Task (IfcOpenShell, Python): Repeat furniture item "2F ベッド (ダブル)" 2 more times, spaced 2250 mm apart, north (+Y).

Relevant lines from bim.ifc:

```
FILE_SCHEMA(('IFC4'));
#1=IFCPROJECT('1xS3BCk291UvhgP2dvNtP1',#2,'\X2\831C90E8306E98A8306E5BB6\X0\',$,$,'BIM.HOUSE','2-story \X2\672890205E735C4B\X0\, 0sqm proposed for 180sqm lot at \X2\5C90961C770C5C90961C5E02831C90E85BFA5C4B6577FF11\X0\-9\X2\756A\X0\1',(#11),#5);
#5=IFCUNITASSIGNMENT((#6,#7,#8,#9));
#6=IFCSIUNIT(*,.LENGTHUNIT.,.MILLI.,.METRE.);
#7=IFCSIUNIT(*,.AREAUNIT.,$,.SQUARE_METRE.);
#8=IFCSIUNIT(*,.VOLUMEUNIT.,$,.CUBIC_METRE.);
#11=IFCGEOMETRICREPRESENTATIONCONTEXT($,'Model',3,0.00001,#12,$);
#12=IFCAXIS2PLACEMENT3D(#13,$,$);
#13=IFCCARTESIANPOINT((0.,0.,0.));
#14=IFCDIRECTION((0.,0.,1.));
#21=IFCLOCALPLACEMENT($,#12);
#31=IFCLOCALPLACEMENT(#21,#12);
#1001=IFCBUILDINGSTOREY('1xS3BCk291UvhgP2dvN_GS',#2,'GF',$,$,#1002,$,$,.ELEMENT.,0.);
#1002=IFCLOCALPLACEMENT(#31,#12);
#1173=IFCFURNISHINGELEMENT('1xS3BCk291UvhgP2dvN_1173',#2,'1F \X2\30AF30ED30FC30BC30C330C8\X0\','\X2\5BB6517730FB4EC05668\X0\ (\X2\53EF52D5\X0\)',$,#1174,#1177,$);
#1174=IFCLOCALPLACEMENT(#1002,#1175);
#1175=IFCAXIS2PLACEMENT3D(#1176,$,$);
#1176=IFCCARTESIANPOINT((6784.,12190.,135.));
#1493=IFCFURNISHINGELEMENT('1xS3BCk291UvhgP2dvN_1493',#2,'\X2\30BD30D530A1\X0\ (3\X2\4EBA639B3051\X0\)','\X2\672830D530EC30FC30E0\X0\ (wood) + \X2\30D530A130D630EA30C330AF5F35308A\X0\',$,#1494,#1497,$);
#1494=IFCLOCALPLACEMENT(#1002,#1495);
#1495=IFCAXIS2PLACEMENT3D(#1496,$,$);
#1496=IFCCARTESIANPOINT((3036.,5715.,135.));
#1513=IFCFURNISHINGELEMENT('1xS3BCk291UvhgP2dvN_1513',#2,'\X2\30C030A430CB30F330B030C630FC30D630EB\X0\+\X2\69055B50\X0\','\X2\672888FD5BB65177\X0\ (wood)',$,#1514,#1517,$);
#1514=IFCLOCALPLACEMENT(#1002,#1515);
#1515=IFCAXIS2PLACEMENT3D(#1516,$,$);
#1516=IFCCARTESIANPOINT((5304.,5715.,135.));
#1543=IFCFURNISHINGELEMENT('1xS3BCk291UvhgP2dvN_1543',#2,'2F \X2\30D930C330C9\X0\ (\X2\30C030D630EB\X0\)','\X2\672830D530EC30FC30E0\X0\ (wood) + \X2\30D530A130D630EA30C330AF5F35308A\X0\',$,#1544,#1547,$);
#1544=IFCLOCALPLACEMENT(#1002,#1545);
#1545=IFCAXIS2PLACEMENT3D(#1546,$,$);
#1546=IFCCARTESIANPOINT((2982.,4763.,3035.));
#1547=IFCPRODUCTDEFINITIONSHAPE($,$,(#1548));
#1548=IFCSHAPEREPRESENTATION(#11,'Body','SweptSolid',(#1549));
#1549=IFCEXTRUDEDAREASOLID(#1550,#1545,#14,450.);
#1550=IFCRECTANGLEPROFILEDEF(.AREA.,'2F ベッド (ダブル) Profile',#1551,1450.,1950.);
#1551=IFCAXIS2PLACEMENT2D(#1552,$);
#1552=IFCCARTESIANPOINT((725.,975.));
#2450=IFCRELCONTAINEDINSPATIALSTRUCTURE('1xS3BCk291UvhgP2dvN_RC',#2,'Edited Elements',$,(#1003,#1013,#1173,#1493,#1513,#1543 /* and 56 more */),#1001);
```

```python
import numpy as np
import ifcopenshell
import ifcopenshell.api.geometry
import ifcopenshell.api.root
import ifcopenshell.util.element
import ifcopenshell.util.placement
import ifcopenshell.util.unit

model = ifcopenshell.open("bim.ifc")
unit_scale = ifcopenshell.util.unit.calculate_unit_scale(model)


def reuse_history(source, copy):
    """copy_class also copies each property set's owner history, people and application; keep the originals."""
    for rel in copy.IsDefinedBy:
        if rel.is_a("IfcRelDefinesByProperties") and (history := rel.RelatingPropertyDefinition.OwnerHistory):
            rel.RelatingPropertyDefinition.OwnerHistory = source.OwnerHistory
            ifcopenshell.util.element.remove_deep2(model, history)


source = model.by_guid("1xS3BCk291UvhgP2dvN_1543")
base = ifcopenshell.util.placement.get_local_placement(source.ObjectPlacement)
step = np.array([0.0, 1.0, 0.0]) * 2.25 / unit_scale

for i in range(1, 3):
    copy = ifcopenshell.api.root.copy_class(model, product=source)
    copy.Representation = ifcopenshell.util.element.copy_deep(
        model, source.Representation, exclude=["IfcGeometricRepresentationContext", "IfcRepresentationMap"]
    )
    reuse_history(source, copy)
    matrix = base.copy()
    matrix[:3, 3] += i * step
    print("added at", matrix[:3, 3].round(3) + 0.0)
    ifcopenshell.api.geometry.edit_object_placement(model, product=copy, matrix=matrix, is_si=False)

model.write("bim_updated.ifc")
```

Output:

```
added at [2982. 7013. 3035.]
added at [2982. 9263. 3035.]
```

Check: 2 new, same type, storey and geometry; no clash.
